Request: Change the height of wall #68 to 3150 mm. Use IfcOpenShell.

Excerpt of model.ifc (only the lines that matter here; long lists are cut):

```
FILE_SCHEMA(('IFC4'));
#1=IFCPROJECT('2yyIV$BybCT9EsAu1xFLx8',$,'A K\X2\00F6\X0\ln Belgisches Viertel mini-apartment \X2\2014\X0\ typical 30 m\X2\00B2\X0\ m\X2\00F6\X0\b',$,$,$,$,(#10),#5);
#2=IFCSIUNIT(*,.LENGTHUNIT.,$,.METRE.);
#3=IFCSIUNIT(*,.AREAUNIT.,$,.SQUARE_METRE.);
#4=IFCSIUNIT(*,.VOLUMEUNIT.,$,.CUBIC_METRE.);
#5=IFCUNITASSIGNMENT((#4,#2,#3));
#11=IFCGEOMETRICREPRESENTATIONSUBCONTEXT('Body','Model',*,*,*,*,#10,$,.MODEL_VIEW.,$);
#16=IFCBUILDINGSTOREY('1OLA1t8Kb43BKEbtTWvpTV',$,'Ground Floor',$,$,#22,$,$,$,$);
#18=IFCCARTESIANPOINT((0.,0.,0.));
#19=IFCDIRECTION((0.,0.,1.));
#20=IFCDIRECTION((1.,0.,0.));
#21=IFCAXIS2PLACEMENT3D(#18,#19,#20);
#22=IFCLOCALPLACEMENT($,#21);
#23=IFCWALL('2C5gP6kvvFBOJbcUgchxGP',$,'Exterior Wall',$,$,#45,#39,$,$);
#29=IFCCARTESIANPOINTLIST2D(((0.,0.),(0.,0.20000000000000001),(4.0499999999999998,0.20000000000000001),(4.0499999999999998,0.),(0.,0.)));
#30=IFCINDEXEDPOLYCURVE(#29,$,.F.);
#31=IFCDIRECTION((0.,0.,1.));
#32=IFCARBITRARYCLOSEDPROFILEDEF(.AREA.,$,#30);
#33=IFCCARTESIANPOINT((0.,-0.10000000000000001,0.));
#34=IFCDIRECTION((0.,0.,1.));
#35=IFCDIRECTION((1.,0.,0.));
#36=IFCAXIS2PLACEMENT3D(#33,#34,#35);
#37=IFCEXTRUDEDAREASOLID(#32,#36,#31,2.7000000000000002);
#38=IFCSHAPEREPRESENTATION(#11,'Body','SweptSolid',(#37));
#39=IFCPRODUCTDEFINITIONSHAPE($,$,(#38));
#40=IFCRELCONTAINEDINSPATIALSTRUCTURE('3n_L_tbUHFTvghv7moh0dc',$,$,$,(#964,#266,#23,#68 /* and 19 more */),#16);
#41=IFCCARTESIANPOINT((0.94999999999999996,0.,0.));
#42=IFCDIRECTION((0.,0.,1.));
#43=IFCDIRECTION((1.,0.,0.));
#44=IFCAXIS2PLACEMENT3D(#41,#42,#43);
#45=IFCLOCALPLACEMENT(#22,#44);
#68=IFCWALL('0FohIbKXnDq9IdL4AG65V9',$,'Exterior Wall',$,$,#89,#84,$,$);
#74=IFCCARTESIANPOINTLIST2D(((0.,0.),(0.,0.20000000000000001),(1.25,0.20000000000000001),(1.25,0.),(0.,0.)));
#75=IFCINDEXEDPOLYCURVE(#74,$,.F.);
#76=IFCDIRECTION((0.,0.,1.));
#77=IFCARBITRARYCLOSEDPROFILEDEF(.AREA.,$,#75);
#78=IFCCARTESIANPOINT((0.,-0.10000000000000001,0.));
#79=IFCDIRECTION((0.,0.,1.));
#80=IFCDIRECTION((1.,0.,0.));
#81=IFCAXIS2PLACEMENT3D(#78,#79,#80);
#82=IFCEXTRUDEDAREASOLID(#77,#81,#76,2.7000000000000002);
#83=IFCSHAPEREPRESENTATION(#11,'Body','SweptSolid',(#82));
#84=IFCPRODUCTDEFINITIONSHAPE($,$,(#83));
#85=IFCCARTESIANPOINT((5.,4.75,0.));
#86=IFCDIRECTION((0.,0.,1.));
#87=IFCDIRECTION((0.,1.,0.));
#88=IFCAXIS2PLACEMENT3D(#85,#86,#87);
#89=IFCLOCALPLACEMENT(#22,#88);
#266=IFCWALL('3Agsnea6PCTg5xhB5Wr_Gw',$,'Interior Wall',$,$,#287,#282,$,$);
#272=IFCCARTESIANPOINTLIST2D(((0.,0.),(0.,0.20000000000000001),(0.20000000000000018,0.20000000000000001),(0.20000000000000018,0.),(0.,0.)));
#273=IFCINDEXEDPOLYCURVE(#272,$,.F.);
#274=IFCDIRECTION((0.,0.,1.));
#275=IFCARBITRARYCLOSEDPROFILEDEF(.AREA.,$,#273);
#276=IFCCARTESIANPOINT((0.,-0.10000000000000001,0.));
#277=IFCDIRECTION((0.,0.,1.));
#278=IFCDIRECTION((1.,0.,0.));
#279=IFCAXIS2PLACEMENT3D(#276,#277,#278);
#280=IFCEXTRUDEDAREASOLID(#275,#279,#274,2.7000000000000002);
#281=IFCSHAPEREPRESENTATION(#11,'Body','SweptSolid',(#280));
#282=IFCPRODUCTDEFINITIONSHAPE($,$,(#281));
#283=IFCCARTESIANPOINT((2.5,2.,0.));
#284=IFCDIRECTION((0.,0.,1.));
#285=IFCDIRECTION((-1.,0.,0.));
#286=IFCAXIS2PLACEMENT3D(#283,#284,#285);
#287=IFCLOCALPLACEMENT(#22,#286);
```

```python
import ifcopenshell
import ifcopenshell.geom
import ifcopenshell.util.representation
import ifcopenshell.util.shape
import ifcopenshell.util.unit

model = ifcopenshell.open("model.ifc")
unit_scale = ifcopenshell.util.unit.calculate_unit_scale(model)
settings = ifcopenshell.geom.settings()


def volume(element):
    """Net volume in cubic metres, openings subtracted."""
    shape = ifcopenshell.geom.create_shape(settings, element)
    return ifcopenshell.util.shape.get_volume(shape.geometry)


wall = model.by_guid("0FohIbKXnDq9IdL4AG65V9")
before = volume(wall)

body = ifcopenshell.util.representation.get_representation(wall, "Model", "Body")
solid = body.Items[0]
old_height = solid.Depth
solid.Depth = 3.15 / unit_scale
after = volume(wall)

print(f"height {old_height:g} -> {solid.Depth:g}, volume {before:.3f} -> {after:.3f} m3")

model.write("model-out.ifc")
```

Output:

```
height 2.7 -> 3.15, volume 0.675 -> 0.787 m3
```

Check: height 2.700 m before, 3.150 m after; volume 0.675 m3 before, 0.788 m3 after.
